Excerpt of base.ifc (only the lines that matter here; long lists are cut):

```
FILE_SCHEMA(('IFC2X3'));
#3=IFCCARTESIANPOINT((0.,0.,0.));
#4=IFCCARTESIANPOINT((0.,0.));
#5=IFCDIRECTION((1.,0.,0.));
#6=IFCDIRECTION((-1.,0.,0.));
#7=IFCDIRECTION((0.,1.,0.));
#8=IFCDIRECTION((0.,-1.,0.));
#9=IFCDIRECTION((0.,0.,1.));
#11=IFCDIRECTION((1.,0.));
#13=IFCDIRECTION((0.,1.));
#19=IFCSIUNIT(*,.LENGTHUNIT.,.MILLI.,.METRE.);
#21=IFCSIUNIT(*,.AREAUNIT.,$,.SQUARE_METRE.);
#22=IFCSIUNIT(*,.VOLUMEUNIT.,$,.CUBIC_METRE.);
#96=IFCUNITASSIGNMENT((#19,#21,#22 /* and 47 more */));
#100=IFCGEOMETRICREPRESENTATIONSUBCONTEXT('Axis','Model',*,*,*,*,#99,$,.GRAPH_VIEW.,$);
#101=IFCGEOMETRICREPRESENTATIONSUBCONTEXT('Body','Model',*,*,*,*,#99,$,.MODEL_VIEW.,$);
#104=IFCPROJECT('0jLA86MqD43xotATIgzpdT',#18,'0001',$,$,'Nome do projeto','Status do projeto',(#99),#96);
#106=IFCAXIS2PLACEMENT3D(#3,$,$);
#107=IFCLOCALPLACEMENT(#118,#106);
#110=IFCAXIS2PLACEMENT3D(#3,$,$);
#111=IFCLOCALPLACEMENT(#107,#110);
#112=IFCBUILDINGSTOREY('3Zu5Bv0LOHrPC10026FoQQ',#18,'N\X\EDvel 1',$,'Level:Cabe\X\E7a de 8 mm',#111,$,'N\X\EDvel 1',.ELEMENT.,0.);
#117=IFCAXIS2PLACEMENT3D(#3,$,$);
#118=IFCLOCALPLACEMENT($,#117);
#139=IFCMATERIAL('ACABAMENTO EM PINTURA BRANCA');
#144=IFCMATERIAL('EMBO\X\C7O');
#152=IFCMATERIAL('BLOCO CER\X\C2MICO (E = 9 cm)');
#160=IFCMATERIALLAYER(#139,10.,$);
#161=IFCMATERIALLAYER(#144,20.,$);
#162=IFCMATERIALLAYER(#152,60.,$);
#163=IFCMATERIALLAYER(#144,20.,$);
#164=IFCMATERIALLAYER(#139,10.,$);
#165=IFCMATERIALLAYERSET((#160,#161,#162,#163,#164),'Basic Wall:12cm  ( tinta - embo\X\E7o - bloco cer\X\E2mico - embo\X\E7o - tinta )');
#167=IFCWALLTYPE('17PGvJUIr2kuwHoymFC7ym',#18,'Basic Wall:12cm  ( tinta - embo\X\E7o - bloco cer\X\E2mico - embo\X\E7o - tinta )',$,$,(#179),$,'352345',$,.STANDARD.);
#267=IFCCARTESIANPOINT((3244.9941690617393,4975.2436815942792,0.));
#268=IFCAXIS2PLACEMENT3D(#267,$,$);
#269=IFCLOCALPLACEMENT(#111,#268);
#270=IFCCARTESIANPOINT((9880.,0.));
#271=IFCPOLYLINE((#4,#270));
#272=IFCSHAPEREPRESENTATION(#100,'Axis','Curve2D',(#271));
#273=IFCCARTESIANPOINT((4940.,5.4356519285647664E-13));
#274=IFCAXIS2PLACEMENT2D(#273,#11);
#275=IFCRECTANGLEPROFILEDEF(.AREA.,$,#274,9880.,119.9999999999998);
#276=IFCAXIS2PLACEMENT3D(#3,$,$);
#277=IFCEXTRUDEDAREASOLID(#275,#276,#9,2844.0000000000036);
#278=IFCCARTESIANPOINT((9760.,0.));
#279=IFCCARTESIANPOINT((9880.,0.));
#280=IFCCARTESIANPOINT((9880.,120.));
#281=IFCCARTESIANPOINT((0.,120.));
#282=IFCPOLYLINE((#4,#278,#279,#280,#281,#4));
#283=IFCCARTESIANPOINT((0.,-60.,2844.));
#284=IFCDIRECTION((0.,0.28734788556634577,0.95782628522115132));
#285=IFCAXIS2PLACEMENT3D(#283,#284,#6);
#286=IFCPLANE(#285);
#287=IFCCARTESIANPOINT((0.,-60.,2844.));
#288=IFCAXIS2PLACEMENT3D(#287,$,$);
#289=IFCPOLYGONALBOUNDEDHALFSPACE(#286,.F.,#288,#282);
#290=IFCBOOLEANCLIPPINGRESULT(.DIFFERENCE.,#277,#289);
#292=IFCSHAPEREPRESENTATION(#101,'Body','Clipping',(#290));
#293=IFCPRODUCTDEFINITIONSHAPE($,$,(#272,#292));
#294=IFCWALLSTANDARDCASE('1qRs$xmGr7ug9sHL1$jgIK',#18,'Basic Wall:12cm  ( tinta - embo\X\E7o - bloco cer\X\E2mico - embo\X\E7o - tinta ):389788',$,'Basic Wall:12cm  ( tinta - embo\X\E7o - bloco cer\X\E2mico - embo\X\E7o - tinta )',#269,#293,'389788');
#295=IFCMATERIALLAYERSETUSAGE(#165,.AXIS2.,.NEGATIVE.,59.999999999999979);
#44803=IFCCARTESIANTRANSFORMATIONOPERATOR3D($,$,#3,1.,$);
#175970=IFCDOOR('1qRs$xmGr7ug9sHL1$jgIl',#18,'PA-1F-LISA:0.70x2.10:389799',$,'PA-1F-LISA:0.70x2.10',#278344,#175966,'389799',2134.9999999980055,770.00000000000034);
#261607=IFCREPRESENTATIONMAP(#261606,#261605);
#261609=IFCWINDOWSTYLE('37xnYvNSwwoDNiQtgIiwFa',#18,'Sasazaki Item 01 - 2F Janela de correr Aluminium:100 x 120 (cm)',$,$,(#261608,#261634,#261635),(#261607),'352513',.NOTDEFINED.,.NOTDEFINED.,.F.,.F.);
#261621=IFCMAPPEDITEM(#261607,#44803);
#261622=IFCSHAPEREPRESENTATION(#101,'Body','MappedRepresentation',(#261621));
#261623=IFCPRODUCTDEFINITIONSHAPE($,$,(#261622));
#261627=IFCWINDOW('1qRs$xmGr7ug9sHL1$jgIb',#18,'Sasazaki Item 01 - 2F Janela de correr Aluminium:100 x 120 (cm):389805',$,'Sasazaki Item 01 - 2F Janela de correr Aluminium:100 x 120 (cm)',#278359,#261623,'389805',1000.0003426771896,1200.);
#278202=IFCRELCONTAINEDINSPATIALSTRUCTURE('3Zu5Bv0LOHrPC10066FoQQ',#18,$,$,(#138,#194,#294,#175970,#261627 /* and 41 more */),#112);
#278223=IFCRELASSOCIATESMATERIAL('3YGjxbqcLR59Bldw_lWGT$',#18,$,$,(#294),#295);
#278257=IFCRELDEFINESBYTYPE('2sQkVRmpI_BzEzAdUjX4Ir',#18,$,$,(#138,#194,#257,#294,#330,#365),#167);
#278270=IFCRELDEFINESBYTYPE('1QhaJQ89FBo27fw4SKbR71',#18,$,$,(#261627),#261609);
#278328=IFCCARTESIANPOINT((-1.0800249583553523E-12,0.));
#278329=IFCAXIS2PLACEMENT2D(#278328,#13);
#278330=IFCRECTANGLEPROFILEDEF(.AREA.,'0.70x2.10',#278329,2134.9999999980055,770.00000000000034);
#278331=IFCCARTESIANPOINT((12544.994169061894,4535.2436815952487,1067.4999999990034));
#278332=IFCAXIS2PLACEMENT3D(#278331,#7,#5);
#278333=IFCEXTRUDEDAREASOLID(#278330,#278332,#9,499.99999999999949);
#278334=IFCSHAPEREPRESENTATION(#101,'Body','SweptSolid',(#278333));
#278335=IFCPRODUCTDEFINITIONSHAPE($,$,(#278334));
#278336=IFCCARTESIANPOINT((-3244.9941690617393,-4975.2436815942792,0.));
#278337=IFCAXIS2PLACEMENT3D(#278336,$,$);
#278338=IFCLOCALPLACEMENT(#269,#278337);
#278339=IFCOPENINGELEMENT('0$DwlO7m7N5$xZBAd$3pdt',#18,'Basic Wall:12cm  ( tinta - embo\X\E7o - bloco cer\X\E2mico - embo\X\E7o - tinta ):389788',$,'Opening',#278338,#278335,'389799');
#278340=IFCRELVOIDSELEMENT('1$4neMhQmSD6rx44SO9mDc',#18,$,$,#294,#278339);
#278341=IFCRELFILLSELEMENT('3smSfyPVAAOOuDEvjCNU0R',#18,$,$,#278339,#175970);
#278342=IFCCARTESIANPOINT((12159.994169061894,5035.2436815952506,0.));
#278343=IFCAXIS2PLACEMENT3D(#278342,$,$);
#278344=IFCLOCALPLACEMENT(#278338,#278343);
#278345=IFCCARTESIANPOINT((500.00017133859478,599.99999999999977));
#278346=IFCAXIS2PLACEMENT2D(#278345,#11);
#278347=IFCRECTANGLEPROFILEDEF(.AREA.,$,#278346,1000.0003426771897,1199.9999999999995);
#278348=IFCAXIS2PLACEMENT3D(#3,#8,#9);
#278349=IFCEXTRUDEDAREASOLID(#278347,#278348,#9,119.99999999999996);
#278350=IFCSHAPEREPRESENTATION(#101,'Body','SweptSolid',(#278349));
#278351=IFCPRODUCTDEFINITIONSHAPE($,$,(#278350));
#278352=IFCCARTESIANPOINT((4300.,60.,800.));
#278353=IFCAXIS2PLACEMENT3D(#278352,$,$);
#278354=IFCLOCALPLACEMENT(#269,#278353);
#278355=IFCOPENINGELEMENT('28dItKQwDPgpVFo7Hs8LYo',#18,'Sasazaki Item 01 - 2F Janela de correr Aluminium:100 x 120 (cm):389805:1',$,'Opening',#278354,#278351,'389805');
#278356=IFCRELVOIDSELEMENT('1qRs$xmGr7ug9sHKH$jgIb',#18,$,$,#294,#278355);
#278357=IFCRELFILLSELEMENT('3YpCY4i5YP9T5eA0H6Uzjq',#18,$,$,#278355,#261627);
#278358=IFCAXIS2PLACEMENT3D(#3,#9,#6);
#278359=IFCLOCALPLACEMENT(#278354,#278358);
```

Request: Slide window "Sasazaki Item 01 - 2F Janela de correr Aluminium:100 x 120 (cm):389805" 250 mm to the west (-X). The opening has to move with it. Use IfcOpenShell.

```python
import ifcopenshell
import ifcopenshell.api.geometry
import ifcopenshell.util.placement
import ifcopenshell.util.unit

model = ifcopenshell.open("base.ifc")
unit_scale = ifcopenshell.util.unit.calculate_unit_scale(model)

window = model.by_id(261627)
opening = window.FillsVoids[0].RelatingOpeningElement
wall = opening.VoidsElements[0].RelatingBuildingElement

wall_matrix = ifcopenshell.util.placement.get_local_placement(wall.ObjectPlacement)
shift = wall_matrix[:3, 0] * -0.25 / unit_scale
before = ifcopenshell.util.placement.get_local_placement(window.ObjectPlacement)[:3, 3].copy()

# The window is placed relative to its opening, so it follows when the opening moves.
matrix = ifcopenshell.util.placement.get_local_placement(opening.ObjectPlacement)
matrix[:3, 3] += shift
ifcopenshell.api.geometry.edit_object_placement(
    model, product=opening, matrix=matrix, is_si=False, should_transform_children=True
)

after = ifcopenshell.util.placement.get_local_placement(window.ObjectPlacement)[:3, 3]
print("window moved by", (after - before).round(3) + 0.0)

model.write("base_edited.ifc")
```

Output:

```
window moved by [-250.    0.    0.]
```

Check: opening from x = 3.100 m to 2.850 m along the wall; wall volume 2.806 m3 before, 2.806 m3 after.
